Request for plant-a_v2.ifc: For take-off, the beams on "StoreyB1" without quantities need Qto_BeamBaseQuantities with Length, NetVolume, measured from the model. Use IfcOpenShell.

First a look at what the model holds.

```python
import ifcopenshell
import ifcopenshell.util.element
import ifcopenshell.util.unit

model = ifcopenshell.open("plant-a_v2.ifc")
print(model.schema)
for unit_type in ("LENGTHUNIT", "AREAUNIT", "VOLUMEUNIT"):
    print(unit_type, ifcopenshell.util.unit.calculate_unit_scale(model, unit_type))
storey = next(s for s in model.by_type("IfcBuildingStorey") if s.Name == "StoreyB1")
beams = [e for e in ifcopenshell.util.element.get_decomposition(storey) if e.is_a("IfcBeam")]
for e in sorted(beams, key=lambda e: e.id()):
    print(e.id(), e.is_a(), e.Name, list(ifcopenshell.util.element.get_psets(e, qtos_only=True)), sep=" | ")
```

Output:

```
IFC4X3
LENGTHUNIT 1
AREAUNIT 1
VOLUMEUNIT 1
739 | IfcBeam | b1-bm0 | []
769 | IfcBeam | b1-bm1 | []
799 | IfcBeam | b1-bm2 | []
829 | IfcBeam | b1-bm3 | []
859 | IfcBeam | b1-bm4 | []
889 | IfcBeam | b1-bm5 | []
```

```python
import ifcopenshell
import ifcopenshell.api.pset
import ifcopenshell.geom
import ifcopenshell.util.element
import ifcopenshell.util.shape
import ifcopenshell.util.unit

model = ifcopenshell.open("plant-a_v2.ifc")
unit_scale = ifcopenshell.util.unit.calculate_unit_scale(model)
volume_scale = ifcopenshell.util.unit.calculate_unit_scale(model, "VOLUMEUNIT")
settings = ifcopenshell.geom.settings()

storey = next(s for s in model.by_type("IfcBuildingStorey") if s.Name == "StoreyB1")
beams = [e for e in ifcopenshell.util.element.get_decomposition(storey) if e.is_a("IfcBeam")]

for e in sorted(beams, key=lambda e: e.id()):
    if ifcopenshell.util.element.get_psets(e, qtos_only=True, should_inherit=False):
        continue
    # Geometry comes back in metres, in the element's own axes.
    shape = ifcopenshell.geom.create_shape(settings, e)
    values = {
        "Length": ifcopenshell.util.shape.get_max_xyz(shape.geometry) / unit_scale,
        "NetVolume": ifcopenshell.util.shape.get_volume(shape.geometry) / volume_scale,
    }
    qto = ifcopenshell.api.pset.add_qto(model, product=e, name="Qto_BeamBaseQuantities")
    ifcopenshell.api.pset.edit_qto(model, qto=qto, properties=values)
    print(e.id(), {k: round(v, 3) for k, v in values.items()})

model.write("plant-a_v2_edited.ifc")
```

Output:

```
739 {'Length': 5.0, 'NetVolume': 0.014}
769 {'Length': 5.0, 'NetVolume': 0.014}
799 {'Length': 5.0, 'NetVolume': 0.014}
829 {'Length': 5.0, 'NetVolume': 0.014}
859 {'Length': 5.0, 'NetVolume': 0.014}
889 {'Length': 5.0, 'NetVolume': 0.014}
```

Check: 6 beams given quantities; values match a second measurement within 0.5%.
